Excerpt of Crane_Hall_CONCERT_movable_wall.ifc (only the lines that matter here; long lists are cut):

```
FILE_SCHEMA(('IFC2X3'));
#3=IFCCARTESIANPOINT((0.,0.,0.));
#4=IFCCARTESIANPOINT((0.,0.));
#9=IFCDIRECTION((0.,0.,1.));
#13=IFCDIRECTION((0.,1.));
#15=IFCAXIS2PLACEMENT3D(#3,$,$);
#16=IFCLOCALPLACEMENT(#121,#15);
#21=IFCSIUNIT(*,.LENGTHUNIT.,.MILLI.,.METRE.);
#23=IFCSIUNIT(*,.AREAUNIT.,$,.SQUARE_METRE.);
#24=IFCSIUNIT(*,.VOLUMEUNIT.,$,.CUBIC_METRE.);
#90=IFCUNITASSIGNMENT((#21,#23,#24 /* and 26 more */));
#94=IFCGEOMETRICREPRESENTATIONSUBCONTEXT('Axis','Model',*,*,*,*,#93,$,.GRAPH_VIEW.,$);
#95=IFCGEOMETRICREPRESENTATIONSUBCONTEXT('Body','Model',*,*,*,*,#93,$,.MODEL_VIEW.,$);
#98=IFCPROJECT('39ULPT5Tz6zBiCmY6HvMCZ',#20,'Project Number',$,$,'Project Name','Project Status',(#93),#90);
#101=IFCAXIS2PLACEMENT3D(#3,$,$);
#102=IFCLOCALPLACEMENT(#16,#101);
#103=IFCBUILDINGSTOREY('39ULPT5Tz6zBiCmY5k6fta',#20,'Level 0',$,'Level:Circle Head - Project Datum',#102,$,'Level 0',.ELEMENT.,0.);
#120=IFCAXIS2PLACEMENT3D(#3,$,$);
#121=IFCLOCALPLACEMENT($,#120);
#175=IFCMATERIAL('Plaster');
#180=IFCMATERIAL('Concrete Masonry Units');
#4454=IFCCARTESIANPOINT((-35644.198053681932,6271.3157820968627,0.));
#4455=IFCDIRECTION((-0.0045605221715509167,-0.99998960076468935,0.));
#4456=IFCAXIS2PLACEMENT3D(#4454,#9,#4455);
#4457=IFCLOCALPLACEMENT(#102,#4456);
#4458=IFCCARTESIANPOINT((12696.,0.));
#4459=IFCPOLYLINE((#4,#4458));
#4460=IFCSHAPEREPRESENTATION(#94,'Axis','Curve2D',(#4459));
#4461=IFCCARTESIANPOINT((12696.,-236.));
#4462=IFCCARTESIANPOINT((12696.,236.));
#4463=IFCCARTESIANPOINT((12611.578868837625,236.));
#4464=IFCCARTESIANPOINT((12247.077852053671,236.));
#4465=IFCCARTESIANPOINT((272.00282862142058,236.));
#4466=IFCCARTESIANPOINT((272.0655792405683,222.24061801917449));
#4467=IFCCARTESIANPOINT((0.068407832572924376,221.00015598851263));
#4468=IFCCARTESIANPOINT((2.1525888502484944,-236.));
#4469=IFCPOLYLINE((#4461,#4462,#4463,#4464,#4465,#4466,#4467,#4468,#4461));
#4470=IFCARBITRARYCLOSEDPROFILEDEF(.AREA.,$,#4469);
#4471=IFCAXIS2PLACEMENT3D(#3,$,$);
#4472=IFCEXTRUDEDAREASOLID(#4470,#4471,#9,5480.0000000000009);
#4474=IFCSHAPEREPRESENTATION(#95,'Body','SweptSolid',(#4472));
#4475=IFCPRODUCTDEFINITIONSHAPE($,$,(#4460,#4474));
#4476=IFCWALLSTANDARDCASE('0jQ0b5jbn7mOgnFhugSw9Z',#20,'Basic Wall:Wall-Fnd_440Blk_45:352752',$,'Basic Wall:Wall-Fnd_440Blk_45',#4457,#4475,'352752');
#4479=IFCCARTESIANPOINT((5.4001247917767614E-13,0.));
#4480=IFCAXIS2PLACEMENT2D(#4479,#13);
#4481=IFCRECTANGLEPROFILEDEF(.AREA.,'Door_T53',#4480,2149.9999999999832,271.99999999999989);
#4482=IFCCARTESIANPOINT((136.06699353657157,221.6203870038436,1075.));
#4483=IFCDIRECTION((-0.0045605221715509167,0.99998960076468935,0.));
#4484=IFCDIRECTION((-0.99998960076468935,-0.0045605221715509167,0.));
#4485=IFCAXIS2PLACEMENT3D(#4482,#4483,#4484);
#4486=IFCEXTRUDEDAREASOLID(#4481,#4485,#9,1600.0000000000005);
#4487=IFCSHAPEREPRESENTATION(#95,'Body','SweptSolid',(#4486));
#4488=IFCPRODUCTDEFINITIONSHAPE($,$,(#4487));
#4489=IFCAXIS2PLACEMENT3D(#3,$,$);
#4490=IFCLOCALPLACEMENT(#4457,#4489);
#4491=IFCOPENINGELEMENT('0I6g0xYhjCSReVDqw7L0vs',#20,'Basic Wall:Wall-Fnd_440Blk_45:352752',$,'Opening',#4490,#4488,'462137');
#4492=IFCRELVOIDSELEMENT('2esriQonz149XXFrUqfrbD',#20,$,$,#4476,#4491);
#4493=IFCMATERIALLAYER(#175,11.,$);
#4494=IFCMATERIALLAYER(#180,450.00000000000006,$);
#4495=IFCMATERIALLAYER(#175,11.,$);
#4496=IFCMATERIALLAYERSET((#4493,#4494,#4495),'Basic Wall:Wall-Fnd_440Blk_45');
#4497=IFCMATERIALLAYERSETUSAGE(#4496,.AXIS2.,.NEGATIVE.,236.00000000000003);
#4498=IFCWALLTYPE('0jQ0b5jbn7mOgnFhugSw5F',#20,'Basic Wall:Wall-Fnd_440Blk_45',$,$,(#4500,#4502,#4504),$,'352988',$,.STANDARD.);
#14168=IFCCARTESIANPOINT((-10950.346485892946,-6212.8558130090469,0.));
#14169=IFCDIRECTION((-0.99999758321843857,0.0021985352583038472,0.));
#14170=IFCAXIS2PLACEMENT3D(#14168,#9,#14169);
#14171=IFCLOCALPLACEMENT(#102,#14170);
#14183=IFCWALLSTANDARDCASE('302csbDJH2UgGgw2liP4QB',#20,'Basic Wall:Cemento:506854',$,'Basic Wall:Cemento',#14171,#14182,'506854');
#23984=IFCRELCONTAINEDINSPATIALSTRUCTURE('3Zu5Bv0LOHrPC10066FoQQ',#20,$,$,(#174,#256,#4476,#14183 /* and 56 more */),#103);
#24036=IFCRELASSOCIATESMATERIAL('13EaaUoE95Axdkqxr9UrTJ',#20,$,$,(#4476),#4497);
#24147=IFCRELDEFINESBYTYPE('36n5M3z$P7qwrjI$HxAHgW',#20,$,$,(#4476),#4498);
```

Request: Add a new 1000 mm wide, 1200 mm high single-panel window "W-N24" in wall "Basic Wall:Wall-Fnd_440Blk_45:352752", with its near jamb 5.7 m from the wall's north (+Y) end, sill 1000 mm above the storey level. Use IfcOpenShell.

```python
import numpy as np
import ifcopenshell
import ifcopenshell.api.feature
import ifcopenshell.api.geometry
import ifcopenshell.api.root
import ifcopenshell.api.spatial
import ifcopenshell.api.type
import ifcopenshell.geom
import ifcopenshell.util.element
import ifcopenshell.util.placement
import ifcopenshell.util.representation
import ifcopenshell.util.shape
import ifcopenshell.util.unit

model = ifcopenshell.open("Crane_Hall_CONCERT_movable_wall.ifc")
unit_scale = ifcopenshell.util.unit.calculate_unit_scale(model)
settings = ifcopenshell.geom.settings()


def volume(element):
    """Net volume in cubic metres, openings subtracted."""
    shape = ifcopenshell.geom.create_shape(settings, element)
    return ifcopenshell.util.shape.get_volume(shape.geometry)


wall = model.by_id(4476)
storey = ifcopenshell.util.element.get_container(wall, ifc_class="IfcBuildingStorey")
context = ifcopenshell.util.representation.get_context(model, "Model", "Body", "MODEL_VIEW")
before = volume(wall)

width, height, from_end, sill = 1, 1.2, 5.7, 1  # metres

# The wall runs along its own X axis, and the end named is its -X end.
wall_shape = ifcopenshell.geom.create_shape(settings, wall)
x, y, z = ifcopenshell.util.shape.get_vertices(wall_shape.geometry).T
start = x.min() + from_end
face, thickness = float(y.min()), float(y.max() - y.min())
wall_matrix = ifcopenshell.util.placement.get_local_placement(wall.ObjectPlacement)
level = ifcopenshell.util.placement.get_local_placement(storey.ObjectPlacement)[2, 3]


def in_wall(x, y):
    """Placement at x, y metres in the wall's axes, at sill height."""
    matrix = wall_matrix.copy()
    matrix[:, 3] = wall_matrix @ np.array([x / unit_scale, y / unit_scale, 0.0, 1.0])
    matrix[2, 3] = level + sill / unit_scale
    return matrix


# Opening: a box that overshoots both wall faces by 50 mm.
opening = ifcopenshell.api.root.create_entity(model, ifc_class="IfcOpeningElement")
box = ifcopenshell.api.geometry.add_wall_representation(
    model, context=context, length=width, height=height, thickness=thickness + 0.1
)
ifcopenshell.api.geometry.assign_representation(model, product=opening, representation=box)
ifcopenshell.api.geometry.edit_object_placement(model, product=opening, matrix=in_wall(start, face - 0.05), is_si=False)
ifcopenshell.api.feature.add_feature(model, feature=opening, element=wall)

window = ifcopenshell.api.root.create_entity(model, ifc_class="IfcWindow", name="W-N24")
window.OverallWidth, window.OverallHeight = width / unit_scale, height / unit_scale
body = ifcopenshell.api.geometry.add_window_representation(
    model,
    context=context,
    overall_width=window.OverallWidth,
    overall_height=window.OverallHeight,
    partition_type="SINGLE_PANEL",
)
ifcopenshell.api.geometry.assign_representation(model, product=window, representation=body)
ifcopenshell.api.spatial.assign_container(model, products=[window], relating_structure=storey)
fills = ifcopenshell.api.feature.add_filling(model, opening=opening, element=window)
fills.OwnerHistory = window.OwnerHistory  # required in IFC2X3

# IFC2X3 keeps the operation on the window style.
style = ifcopenshell.api.root.create_entity(model, ifc_class="IfcWindowStyle", name="W-N24")
style.OperationType, style.ConstructionType = "SINGLE_PANEL", "NOTDEFINED"
style.ParameterTakesPrecedence = style.Sizeable = False
ifcopenshell.api.type.assign_type(model, related_objects=[window], relating_type=style)

# Centre the window in the wall's thickness.
ifcopenshell.api.geometry.edit_object_placement(model, product=window, matrix=in_wall(start, face), is_si=False)
window_shape = ifcopenshell.geom.create_shape(settings, window)
depth = ifcopenshell.util.shape.get_vertices(window_shape.geometry)[:, 1]
offset = face + thickness / 2 - (depth.min() + depth.max()) / 2
ifcopenshell.api.geometry.edit_object_placement(model, product=window, matrix=in_wall(start, offset), is_si=False)

after = volume(wall)

print(f"wall volume {before:.3f} -> {after:.3f} m3")

model.write("Crane_Hall_CONCERT_movable_wall-out.ifc")
```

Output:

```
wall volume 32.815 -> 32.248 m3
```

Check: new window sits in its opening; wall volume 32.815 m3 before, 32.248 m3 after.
